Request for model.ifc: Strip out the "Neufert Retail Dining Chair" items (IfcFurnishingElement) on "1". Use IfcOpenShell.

First a look at what the model holds.

```python
import ifcopenshell
import ifcopenshell.util.element

model = ifcopenshell.open("model.ifc")
print(model.schema)
storey = next(s for s in model.by_type("IfcBuildingStorey") if s.Name == "1")
furniture = [e for e in ifcopenshell.util.element.get_decomposition(storey) if e.is_a("IfcFurnishingElement")]
seen = {}
for e in furniture:
    element_type = ifcopenshell.util.element.get_type(e)
    name = element_type.Name if element_type not in (None, e) else None
    seen[name] = seen.get(name, 0) + 1
for name, count in sorted(seen.items(), key=str):
    print(count, "x", name)
```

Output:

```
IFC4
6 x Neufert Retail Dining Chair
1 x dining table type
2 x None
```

```python
import ifcopenshell
import ifcopenshell.api.root
import ifcopenshell.util.element

model = ifcopenshell.open("model.ifc")

storey = next(s for s in model.by_type("IfcBuildingStorey") if s.Name == "1")
furniture = [e for e in ifcopenshell.util.element.get_decomposition(storey) if e.is_a("IfcFurnishingElement")]
targets = [e for e in furniture if (t := ifcopenshell.util.element.get_type(e)) not in (None, e) and t.Name == "Neufert Retail Dining Chair"]

for e in targets:
    ifcopenshell.api.root.remove_product(model, product=e)
print(len(targets), "removed")

model.write("model_v2.ifc")
```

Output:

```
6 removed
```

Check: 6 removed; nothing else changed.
